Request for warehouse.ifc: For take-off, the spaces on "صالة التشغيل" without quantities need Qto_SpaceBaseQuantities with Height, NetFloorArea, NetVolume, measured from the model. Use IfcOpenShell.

First a look at what the model holds.

```python
import ifcopenshell
import ifcopenshell.util.element
import ifcopenshell.util.unit

model = ifcopenshell.open("warehouse.ifc")
print(model.schema)
for unit_type in ("LENGTHUNIT", "AREAUNIT", "VOLUMEUNIT"):
    print(unit_type, ifcopenshell.util.unit.calculate_unit_scale(model, unit_type))
storey = next(s for s in model.by_type("IfcBuildingStorey") if s.Name == "صالة التشغيل")
spaces = [e for e in ifcopenshell.util.element.get_decomposition(storey) if e.is_a("IfcSpace")]
for e in sorted(spaces, key=lambda e: e.id()):
    print(e.id(), e.is_a(), e.Name, list(ifcopenshell.util.element.get_psets(e, qtos_only=True)), sep=" | ")
```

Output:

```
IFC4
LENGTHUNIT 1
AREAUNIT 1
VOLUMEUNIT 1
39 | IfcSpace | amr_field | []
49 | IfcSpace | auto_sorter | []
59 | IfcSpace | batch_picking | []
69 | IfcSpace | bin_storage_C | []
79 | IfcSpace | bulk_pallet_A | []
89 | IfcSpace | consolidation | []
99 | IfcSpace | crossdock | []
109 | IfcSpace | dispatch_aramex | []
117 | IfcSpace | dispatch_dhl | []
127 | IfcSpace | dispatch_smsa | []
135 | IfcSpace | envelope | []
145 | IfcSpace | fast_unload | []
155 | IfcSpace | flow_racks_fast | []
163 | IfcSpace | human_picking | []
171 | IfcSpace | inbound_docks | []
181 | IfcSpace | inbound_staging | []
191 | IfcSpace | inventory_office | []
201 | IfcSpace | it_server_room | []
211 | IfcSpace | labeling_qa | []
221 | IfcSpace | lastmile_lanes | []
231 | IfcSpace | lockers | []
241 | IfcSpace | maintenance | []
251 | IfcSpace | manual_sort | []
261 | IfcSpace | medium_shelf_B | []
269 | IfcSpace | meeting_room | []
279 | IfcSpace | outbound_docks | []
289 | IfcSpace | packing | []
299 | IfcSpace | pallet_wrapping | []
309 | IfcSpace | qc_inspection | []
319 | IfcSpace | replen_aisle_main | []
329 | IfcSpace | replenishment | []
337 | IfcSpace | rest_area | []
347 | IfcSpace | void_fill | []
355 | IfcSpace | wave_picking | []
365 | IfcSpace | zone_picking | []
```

```python
import ifcopenshell
import ifcopenshell.api.pset
import ifcopenshell.geom
import ifcopenshell.util.element
import ifcopenshell.util.shape
import ifcopenshell.util.unit

model = ifcopenshell.open("warehouse.ifc")
unit_scale = ifcopenshell.util.unit.calculate_unit_scale(model)
area_scale = ifcopenshell.util.unit.calculate_unit_scale(model, "AREAUNIT")
volume_scale = ifcopenshell.util.unit.calculate_unit_scale(model, "VOLUMEUNIT")
settings = ifcopenshell.geom.settings()

storey = next(s for s in model.by_type("IfcBuildingStorey") if s.Name == "صالة التشغيل")
spaces = [e for e in ifcopenshell.util.element.get_decomposition(storey) if e.is_a("IfcSpace")]

for e in sorted(spaces, key=lambda e: e.id()):
    if ifcopenshell.util.element.get_psets(e, qtos_only=True, should_inherit=False):
        continue
    # Geometry comes back in metres, in the element's own axes.
    shape = ifcopenshell.geom.create_shape(settings, e)
    values = {
        "Height": ifcopenshell.util.shape.get_z(shape.geometry) / unit_scale,
        "NetFloorArea": ifcopenshell.util.shape.get_footprint_area(shape.geometry) / area_scale,
        "NetVolume": ifcopenshell.util.shape.get_volume(shape.geometry) / volume_scale,
    }
    qto = ifcopenshell.api.pset.add_qto(model, product=e, name="Qto_SpaceBaseQuantities")
    ifcopenshell.api.pset.edit_qto(model, qto=qto, properties=values)
    print(e.id(), {k: round(v, 3) for k, v in values.items()})

model.write("warehouse-out.ifc")
```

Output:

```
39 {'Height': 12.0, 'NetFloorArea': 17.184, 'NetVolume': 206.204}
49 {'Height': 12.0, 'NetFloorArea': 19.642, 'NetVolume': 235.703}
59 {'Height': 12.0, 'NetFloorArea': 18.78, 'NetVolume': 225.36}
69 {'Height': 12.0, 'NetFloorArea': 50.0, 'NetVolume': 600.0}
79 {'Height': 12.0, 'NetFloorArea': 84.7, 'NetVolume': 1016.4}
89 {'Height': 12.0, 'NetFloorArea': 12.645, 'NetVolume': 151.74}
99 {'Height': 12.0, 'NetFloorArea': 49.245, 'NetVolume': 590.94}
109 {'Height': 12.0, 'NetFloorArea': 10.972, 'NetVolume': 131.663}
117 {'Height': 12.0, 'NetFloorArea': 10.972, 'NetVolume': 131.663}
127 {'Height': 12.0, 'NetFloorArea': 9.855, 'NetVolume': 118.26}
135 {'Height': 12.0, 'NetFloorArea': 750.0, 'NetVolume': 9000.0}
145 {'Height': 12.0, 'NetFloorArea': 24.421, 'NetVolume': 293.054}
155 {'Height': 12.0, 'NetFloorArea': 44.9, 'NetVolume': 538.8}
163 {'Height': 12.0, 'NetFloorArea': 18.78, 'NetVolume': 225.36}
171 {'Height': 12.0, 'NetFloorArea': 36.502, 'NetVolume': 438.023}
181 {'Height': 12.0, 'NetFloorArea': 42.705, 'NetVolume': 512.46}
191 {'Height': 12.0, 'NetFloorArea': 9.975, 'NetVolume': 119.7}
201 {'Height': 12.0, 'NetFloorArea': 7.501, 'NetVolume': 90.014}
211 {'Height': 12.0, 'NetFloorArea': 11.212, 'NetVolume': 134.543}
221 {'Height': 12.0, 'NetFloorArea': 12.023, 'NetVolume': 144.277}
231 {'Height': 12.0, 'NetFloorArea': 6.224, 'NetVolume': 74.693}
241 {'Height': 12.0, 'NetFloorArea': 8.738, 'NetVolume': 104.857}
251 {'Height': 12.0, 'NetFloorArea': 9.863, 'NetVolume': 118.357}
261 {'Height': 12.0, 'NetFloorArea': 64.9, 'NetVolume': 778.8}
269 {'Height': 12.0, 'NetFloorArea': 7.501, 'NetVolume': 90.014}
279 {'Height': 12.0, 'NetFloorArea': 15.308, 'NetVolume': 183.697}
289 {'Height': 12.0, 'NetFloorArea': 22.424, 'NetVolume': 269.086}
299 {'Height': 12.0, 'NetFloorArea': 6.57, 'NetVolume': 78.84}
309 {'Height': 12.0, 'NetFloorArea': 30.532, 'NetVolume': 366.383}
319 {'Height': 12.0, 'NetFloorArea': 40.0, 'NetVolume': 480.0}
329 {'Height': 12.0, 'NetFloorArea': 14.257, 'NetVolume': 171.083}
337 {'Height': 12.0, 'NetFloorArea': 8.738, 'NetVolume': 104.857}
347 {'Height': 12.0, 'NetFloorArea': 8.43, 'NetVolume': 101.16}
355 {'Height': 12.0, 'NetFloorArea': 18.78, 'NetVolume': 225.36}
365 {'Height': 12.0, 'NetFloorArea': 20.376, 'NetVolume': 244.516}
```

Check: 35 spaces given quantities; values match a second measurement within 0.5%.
